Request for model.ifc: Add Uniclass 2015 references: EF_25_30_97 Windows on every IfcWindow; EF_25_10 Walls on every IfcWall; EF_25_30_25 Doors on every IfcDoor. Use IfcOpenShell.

First a look at what the model holds.

```python
import ifcopenshell

model = ifcopenshell.open("model.ifc")
print(model.schema)
print("classifications:", [c.Name for c in model.by_type("IfcClassification")])
for ifc_class in ("IfcDoor", "IfcRoof", "IfcStair", "IfcWall", "IfcWindow"):
    print(ifc_class, len(model.by_type(ifc_class)))
```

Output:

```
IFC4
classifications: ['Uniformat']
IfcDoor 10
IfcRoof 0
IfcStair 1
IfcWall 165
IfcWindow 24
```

```python
import ifcopenshell
import ifcopenshell.api.classification

model = ifcopenshell.open("model.ifc")

system = ifcopenshell.api.classification.add_classification(model, classification="Uniclass 2015")

codes = {
    "IfcWindow": ("EF_25_30_97", "Windows"),
    "IfcWall": ("EF_25_10", "Walls"),
    "IfcDoor": ("EF_25_30_25", "Doors"),
}
for ifc_class, (code, name) in codes.items():
    products = model.by_type(ifc_class)
    ifcopenshell.api.classification.add_reference(
        model, products=products, classification=system, identification=code, name=name
    )
    print(code, len(products))

model.write("model_edited.ifc")
```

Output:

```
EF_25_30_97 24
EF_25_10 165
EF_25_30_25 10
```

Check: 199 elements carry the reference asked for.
